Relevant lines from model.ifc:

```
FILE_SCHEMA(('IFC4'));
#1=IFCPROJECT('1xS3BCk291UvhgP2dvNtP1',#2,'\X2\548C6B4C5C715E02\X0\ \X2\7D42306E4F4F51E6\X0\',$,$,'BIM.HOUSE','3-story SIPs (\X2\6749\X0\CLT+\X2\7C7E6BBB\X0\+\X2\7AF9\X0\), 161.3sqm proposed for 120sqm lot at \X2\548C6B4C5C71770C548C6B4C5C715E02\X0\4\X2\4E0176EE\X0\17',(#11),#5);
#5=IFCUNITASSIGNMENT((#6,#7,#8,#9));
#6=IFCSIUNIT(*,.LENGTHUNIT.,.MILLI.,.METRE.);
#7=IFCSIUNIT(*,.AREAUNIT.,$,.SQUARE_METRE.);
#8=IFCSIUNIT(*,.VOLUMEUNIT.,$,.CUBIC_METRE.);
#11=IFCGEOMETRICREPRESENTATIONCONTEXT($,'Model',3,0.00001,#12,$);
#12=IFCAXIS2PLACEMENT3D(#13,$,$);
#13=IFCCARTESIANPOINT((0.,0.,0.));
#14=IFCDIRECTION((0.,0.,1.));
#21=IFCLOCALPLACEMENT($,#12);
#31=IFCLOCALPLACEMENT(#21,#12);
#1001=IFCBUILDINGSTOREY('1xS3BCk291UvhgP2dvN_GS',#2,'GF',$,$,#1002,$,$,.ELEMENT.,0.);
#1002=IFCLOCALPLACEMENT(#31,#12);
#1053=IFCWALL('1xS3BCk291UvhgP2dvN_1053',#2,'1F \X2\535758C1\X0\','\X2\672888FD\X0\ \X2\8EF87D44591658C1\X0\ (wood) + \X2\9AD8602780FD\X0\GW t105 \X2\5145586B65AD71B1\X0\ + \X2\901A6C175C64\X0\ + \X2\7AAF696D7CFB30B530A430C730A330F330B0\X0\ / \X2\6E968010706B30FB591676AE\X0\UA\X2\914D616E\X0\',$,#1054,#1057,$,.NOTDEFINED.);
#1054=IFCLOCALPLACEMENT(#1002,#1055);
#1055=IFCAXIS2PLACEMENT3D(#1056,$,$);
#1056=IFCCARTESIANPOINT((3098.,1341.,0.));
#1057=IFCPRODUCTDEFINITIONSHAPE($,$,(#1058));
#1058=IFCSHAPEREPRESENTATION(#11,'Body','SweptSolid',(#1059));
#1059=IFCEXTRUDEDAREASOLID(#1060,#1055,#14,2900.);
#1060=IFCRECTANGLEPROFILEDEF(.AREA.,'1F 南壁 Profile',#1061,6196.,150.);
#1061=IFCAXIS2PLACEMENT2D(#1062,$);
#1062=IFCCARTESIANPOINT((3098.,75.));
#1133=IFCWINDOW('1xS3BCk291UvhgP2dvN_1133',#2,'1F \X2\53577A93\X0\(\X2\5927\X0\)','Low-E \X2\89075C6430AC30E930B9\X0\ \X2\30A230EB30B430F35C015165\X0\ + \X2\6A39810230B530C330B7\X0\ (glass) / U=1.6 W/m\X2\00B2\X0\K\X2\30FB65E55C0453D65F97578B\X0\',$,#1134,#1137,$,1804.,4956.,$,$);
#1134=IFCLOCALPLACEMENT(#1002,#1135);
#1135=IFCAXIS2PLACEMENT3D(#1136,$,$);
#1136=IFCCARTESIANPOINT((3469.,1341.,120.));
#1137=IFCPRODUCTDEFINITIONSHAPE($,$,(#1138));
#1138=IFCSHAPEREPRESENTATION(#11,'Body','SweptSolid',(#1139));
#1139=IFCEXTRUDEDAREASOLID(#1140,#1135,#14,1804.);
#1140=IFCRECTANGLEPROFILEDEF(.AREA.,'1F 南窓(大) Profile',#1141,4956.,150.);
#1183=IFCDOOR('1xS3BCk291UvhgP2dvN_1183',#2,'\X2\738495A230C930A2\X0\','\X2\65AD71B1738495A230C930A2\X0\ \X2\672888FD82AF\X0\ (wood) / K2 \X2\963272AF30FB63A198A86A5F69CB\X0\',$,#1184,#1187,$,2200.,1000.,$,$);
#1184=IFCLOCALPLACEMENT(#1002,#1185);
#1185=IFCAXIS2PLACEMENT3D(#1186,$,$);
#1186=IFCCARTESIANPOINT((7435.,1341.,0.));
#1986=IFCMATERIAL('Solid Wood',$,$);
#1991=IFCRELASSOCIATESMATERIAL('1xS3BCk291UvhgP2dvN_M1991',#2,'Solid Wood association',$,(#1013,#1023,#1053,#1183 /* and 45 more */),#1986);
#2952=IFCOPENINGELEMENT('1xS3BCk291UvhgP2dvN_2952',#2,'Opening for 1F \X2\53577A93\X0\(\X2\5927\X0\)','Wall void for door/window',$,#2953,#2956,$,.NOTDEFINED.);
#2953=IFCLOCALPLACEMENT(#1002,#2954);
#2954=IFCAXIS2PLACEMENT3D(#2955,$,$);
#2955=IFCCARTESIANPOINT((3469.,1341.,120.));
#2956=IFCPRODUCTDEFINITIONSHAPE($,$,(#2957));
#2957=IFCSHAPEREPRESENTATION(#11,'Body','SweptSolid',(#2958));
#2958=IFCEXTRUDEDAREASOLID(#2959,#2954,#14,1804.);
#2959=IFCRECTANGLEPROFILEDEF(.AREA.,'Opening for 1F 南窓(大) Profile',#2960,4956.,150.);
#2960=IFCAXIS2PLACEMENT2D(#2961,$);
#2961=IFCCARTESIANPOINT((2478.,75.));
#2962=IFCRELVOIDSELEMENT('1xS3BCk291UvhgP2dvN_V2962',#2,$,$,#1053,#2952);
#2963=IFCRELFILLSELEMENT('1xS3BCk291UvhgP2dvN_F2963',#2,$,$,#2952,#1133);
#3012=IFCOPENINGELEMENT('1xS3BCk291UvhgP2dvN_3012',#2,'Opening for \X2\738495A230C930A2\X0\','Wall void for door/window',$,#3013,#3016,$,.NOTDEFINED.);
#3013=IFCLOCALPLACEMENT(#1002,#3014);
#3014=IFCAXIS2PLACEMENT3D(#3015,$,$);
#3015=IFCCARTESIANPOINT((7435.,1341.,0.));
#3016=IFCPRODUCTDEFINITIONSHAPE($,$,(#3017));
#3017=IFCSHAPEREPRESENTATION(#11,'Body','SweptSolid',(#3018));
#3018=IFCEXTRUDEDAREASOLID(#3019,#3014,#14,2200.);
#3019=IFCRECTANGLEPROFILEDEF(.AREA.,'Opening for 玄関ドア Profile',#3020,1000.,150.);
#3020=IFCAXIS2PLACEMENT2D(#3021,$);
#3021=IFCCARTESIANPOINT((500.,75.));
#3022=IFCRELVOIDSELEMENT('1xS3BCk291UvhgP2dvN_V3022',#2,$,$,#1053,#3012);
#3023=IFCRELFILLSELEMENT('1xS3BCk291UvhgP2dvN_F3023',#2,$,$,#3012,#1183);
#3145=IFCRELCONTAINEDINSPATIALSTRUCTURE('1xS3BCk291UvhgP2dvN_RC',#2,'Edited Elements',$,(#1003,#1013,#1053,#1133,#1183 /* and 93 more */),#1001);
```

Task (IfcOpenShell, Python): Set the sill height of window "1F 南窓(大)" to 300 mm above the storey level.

```python
import numpy as np
import ifcopenshell
import ifcopenshell.api.geometry
import ifcopenshell.geom
import ifcopenshell.util.element
import ifcopenshell.util.placement
import ifcopenshell.util.shape
import ifcopenshell.util.unit

model = ifcopenshell.open("model.ifc")
unit_scale = ifcopenshell.util.unit.calculate_unit_scale(model)

window = model.by_guid("1xS3BCk291UvhgP2dvN_1133")
opening = window.FillsVoids[0].RelatingOpeningElement
storey = ifcopenshell.util.element.get_container(window, ifc_class="IfcBuildingStorey")
level = ifcopenshell.util.placement.get_local_placement(storey.ObjectPlacement)[2, 3]

# The opening's origin need not be at the sill, so measure its lowest point.
shape = ifcopenshell.geom.create_shape(ifcopenshell.geom.settings(), opening)
bottom = ifcopenshell.util.shape.get_shape_bottom_elevation(shape, shape.geometry) / unit_scale
dz = level + 300.0 - bottom

shift = np.array([0.0, 0.0, dz])
# The window is not placed relative to its opening, so move both.
for product in (opening, window):
    matrix = ifcopenshell.util.placement.get_local_placement(product.ObjectPlacement)
    matrix[:3, 3] += shift
    ifcopenshell.api.geometry.edit_object_placement(model, product=product, matrix=matrix, is_si=False)

print(f"moved by {dz * unit_scale:+.3f} m")

model.write("model_v2.ifc")
```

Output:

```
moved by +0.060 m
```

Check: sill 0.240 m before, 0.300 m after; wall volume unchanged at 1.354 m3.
